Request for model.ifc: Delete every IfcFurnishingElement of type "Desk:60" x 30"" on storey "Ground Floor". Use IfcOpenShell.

First a look at what the model holds.

```python
import ifcopenshell
import ifcopenshell.util.element

model = ifcopenshell.open("model.ifc")
print(model.schema)
storey = next(s for s in model.by_type("IfcBuildingStorey") if s.Name == "Ground Floor")
furniture = [e for e in ifcopenshell.util.element.get_decomposition(storey) if e.is_a("IfcFurnishingElement")]
seen = {}
for e in furniture:
    element_type = ifcopenshell.util.element.get_type(e)
    name = element_type.Name if element_type not in (None, e) else None
    seen[name] = seen.get(name, 0) + 1
for name, count in sorted(seen.items(), key=str):
    print(count, "x", name)
```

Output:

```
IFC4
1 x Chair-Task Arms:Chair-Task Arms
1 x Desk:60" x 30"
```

```python
import ifcopenshell
import ifcopenshell.api.root
import ifcopenshell.util.element

model = ifcopenshell.open("model.ifc")

storey = next(s for s in model.by_type("IfcBuildingStorey") if s.Name == "Ground Floor")
furniture = [e for e in ifcopenshell.util.element.get_decomposition(storey) if e.is_a("IfcFurnishingElement")]
targets = [e for e in furniture if (t := ifcopenshell.util.element.get_type(e)) not in (None, e) and t.Name == 'Desk:60" x 30"']

for e in targets:
    ifcopenshell.api.root.remove_product(model, product=e)
print(len(targets), "removed")

model.write("model_updated.ifc")
```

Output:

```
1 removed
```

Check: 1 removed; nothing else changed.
